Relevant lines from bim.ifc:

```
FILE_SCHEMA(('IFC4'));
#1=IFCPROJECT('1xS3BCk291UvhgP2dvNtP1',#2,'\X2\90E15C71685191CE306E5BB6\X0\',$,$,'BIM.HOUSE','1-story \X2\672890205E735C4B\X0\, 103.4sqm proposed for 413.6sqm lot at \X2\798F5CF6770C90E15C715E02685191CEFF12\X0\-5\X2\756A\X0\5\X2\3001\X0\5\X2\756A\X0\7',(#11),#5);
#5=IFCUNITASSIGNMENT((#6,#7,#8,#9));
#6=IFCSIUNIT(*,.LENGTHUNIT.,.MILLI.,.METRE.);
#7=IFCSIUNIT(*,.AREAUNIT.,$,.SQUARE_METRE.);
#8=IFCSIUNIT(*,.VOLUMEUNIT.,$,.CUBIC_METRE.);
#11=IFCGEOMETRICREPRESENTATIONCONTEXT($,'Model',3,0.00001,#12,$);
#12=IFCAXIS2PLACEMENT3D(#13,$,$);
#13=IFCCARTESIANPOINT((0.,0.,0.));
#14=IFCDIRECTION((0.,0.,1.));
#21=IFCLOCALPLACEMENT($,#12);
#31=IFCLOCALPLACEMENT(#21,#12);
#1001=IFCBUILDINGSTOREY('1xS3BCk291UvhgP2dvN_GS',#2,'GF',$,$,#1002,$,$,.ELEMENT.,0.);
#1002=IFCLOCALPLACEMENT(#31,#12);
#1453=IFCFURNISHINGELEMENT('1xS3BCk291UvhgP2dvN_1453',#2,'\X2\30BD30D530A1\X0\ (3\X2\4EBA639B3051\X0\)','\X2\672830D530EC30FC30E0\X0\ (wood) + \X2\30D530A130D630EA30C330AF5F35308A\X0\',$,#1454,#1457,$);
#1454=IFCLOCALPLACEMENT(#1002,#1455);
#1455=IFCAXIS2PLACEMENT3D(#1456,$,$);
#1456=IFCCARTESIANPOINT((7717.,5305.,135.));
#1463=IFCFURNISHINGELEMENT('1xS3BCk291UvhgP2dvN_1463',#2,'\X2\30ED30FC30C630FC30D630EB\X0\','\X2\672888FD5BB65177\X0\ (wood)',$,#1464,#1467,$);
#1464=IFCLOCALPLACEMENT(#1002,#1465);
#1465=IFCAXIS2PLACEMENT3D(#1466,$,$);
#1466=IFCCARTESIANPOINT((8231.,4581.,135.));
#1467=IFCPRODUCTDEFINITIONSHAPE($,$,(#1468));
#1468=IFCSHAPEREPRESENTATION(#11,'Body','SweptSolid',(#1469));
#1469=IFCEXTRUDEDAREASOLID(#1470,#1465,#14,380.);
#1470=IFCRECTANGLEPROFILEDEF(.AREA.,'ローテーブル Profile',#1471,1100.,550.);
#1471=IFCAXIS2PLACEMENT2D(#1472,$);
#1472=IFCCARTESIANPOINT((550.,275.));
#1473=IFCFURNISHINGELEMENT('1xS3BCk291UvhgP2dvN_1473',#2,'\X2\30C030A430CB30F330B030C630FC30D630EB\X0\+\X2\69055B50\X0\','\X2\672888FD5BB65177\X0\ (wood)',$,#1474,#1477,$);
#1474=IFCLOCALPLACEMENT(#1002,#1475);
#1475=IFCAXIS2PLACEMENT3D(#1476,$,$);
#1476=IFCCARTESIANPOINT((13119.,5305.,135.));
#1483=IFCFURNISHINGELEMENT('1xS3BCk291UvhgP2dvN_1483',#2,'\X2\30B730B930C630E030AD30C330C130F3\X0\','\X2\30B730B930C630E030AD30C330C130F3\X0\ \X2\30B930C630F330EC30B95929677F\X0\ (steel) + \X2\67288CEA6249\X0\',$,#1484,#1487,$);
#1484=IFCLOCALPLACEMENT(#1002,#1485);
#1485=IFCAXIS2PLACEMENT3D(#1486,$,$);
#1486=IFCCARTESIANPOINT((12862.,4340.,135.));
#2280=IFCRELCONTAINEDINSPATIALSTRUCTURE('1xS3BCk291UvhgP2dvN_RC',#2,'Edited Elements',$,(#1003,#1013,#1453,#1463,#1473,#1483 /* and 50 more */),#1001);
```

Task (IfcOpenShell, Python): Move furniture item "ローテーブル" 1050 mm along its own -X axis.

```python
import ifcopenshell
import ifcopenshell.api.geometry
import ifcopenshell.util.placement
import ifcopenshell.util.unit

model = ifcopenshell.open("bim.ifc")
unit_scale = ifcopenshell.util.unit.calculate_unit_scale(model)

item = model.by_guid("1xS3BCk291UvhgP2dvN_1463")
matrix = ifcopenshell.util.placement.get_local_placement(item.ObjectPlacement)
matrix[:3, 3] -= matrix[:3, 0] * 1.05 / unit_scale
ifcopenshell.api.geometry.edit_object_placement(model, product=item, matrix=matrix, is_si=False)

print(ifcopenshell.util.placement.get_local_placement(item.ObjectPlacement).round(3) + 0.0)

model.write("bim_updated.ifc")
```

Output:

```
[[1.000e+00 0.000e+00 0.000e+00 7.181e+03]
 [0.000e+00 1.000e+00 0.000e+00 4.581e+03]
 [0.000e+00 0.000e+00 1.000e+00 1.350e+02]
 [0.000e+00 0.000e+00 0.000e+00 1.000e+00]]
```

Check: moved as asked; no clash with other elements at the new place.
